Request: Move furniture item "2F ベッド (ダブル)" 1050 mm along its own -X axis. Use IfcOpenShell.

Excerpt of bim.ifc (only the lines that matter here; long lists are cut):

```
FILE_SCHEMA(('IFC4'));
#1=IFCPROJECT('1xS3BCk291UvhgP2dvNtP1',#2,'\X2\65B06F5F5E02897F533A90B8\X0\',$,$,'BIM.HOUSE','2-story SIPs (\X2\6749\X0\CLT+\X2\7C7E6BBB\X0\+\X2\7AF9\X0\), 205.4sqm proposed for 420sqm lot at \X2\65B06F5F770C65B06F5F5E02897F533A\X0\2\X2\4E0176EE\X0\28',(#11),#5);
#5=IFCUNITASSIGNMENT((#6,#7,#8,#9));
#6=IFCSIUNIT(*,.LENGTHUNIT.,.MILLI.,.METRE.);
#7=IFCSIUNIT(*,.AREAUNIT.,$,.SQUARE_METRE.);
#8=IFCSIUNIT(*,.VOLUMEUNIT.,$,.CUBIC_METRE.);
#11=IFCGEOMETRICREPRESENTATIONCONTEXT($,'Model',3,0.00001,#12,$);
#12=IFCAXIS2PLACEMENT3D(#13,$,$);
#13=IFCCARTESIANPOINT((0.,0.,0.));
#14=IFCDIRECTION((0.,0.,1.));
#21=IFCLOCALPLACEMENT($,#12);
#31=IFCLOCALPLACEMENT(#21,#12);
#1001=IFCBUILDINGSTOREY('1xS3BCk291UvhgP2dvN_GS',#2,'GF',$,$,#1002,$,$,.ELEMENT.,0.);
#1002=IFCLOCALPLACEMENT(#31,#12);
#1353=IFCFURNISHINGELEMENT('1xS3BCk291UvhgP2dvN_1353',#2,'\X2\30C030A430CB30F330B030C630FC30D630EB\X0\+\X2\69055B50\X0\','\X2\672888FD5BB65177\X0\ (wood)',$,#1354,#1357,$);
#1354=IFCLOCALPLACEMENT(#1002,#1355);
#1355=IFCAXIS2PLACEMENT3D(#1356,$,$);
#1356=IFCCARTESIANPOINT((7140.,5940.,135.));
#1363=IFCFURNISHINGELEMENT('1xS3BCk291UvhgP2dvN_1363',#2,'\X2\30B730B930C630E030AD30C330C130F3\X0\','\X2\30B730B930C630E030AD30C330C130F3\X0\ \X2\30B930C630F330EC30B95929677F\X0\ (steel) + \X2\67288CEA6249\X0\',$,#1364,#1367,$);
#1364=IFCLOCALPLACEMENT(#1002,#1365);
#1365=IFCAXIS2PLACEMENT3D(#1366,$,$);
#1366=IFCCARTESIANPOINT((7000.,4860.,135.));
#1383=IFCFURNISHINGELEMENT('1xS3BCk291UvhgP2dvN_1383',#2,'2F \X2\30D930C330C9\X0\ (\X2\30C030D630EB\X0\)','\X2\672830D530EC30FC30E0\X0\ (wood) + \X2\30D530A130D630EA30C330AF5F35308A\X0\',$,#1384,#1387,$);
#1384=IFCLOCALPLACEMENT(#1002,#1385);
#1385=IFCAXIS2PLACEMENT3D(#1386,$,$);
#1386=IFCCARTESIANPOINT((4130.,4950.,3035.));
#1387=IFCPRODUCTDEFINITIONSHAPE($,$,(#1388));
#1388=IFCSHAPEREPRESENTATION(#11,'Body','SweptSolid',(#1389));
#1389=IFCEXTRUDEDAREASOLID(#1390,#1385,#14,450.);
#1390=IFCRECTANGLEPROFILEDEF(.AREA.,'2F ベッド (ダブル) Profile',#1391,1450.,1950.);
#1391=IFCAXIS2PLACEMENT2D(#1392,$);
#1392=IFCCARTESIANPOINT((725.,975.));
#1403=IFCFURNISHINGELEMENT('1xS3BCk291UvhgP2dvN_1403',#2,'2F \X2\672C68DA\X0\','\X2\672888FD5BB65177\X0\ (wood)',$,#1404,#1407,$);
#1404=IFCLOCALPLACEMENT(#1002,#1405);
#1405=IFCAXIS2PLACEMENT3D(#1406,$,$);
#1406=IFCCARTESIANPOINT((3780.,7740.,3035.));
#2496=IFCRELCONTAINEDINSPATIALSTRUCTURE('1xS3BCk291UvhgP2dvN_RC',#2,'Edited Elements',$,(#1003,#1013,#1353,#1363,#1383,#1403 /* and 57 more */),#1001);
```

```python
import ifcopenshell
import ifcopenshell.api.geometry
import ifcopenshell.util.placement

model = ifcopenshell.open("bim.ifc")

item = model.by_guid("1xS3BCk291UvhgP2dvN_1383")
matrix = ifcopenshell.util.placement.get_local_placement(item.ObjectPlacement)
matrix[:3, 3] -= matrix[:3, 0] * 1050.0
ifcopenshell.api.geometry.edit_object_placement(model, product=item, matrix=matrix, is_si=False)

print(ifcopenshell.util.placement.get_local_placement(item.ObjectPlacement).round(3) + 0.0)

model.write("bim_v2.ifc")
```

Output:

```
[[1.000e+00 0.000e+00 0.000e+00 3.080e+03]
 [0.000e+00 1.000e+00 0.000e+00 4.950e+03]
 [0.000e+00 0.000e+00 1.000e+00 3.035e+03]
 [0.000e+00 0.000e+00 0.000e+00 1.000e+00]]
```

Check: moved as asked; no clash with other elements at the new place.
